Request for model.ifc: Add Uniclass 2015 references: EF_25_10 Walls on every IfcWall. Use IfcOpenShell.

First a look at what the model holds.

```python
import ifcopenshell

model = ifcopenshell.open("model.ifc")
print(model.schema)
print("classifications:", [c.Name for c in model.by_type("IfcClassification")])
for ifc_class in ("IfcDoor", "IfcRoof", "IfcStair", "IfcWall", "IfcWindow"):
    print(ifc_class, len(model.by_type(ifc_class)))
```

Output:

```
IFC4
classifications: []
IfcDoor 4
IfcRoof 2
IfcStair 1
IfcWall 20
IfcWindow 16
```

```python
import ifcopenshell
import ifcopenshell.api.classification

model = ifcopenshell.open("model.ifc")

system = ifcopenshell.api.classification.add_classification(model, classification="Uniclass 2015")

codes = {
    "IfcWall": ("EF_25_10", "Walls"),
}
for ifc_class, (code, name) in codes.items():
    products = model.by_type(ifc_class)
    ifcopenshell.api.classification.add_reference(
        model, products=products, classification=system, identification=code, name=name
    )
    print(code, len(products))

model.write("model_edited.ifc")
```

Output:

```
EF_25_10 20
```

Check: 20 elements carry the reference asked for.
